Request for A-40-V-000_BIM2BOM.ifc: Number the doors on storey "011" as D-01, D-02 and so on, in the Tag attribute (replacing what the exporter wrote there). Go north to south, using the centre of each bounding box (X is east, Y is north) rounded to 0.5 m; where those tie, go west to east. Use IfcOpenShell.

First a look at what the model holds.

```python
import ifcopenshell
import ifcopenshell.util.element
import ifcopenshell.util.placement

model = ifcopenshell.open("A-40-V-000_BIM2BOM.ifc")
print(model.schema)
storey = next(s for s in model.by_type("IfcBuildingStorey") if s.Name == "011")
doors = [e for e in ifcopenshell.util.element.get_decomposition(storey) if e.is_a("IfcDoor")]
for e in sorted(doors, key=lambda e: e.id()):
    origin = ifcopenshell.util.placement.get_local_placement(e.ObjectPlacement)[:3, 3]
    print(e.id(), e.Tag, e.Name, origin.round(2) + 0.0, sep=" | ")
```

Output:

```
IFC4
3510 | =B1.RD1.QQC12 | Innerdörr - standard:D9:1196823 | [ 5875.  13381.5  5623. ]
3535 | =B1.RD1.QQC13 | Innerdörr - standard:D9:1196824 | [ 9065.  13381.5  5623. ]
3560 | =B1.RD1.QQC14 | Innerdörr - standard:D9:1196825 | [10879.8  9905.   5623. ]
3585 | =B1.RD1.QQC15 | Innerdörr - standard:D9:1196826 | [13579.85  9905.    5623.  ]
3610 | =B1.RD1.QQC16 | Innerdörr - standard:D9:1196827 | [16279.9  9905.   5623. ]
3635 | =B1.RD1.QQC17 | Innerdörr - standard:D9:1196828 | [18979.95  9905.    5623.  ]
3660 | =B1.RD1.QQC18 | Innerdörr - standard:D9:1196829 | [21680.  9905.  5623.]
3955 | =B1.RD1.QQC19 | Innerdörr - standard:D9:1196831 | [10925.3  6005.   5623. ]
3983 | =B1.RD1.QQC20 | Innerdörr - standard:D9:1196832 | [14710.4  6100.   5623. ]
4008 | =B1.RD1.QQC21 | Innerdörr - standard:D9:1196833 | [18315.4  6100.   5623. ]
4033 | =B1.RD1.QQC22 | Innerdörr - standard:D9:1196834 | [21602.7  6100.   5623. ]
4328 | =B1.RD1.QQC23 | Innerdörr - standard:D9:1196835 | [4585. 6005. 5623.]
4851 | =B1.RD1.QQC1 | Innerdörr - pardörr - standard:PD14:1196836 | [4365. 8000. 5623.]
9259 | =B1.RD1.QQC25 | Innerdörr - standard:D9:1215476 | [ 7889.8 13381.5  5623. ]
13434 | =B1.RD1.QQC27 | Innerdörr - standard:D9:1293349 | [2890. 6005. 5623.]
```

```python
import ifcopenshell
import ifcopenshell.geom
import ifcopenshell.util.element
import ifcopenshell.util.shape

model = ifcopenshell.open("A-40-V-000_BIM2BOM.ifc")
settings = ifcopenshell.geom.settings()
settings.set("use-world-coords", True)


def centre(element):
    shape = ifcopenshell.geom.create_shape(settings, element)
    return ifcopenshell.util.shape.get_bbox_centroid(shape.geometry)


storey = next(s for s in model.by_type("IfcBuildingStorey") if s.Name == "011")
doors = [e for e in ifcopenshell.util.element.get_decomposition(storey) if e.is_a("IfcDoor")]

# Insertion points can sit at a corner or the storey origin, so sort by the geometry (in metres).
centres = {e: centre(e) for e in doors}
doors.sort(key=lambda e: (-round(centres[e][1] / 0.5), centres[e][0]))

for i, e in enumerate(doors, start=1):
    number = f"D-{i:02d}"
    e.Tag = number
    print(e.id(), number)

model.write("A-40-V-000_BIM2BOM_edited.ifc")
```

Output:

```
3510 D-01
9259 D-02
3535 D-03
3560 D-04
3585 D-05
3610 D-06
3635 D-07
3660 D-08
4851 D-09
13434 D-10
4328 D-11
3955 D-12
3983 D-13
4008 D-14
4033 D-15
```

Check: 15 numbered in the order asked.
